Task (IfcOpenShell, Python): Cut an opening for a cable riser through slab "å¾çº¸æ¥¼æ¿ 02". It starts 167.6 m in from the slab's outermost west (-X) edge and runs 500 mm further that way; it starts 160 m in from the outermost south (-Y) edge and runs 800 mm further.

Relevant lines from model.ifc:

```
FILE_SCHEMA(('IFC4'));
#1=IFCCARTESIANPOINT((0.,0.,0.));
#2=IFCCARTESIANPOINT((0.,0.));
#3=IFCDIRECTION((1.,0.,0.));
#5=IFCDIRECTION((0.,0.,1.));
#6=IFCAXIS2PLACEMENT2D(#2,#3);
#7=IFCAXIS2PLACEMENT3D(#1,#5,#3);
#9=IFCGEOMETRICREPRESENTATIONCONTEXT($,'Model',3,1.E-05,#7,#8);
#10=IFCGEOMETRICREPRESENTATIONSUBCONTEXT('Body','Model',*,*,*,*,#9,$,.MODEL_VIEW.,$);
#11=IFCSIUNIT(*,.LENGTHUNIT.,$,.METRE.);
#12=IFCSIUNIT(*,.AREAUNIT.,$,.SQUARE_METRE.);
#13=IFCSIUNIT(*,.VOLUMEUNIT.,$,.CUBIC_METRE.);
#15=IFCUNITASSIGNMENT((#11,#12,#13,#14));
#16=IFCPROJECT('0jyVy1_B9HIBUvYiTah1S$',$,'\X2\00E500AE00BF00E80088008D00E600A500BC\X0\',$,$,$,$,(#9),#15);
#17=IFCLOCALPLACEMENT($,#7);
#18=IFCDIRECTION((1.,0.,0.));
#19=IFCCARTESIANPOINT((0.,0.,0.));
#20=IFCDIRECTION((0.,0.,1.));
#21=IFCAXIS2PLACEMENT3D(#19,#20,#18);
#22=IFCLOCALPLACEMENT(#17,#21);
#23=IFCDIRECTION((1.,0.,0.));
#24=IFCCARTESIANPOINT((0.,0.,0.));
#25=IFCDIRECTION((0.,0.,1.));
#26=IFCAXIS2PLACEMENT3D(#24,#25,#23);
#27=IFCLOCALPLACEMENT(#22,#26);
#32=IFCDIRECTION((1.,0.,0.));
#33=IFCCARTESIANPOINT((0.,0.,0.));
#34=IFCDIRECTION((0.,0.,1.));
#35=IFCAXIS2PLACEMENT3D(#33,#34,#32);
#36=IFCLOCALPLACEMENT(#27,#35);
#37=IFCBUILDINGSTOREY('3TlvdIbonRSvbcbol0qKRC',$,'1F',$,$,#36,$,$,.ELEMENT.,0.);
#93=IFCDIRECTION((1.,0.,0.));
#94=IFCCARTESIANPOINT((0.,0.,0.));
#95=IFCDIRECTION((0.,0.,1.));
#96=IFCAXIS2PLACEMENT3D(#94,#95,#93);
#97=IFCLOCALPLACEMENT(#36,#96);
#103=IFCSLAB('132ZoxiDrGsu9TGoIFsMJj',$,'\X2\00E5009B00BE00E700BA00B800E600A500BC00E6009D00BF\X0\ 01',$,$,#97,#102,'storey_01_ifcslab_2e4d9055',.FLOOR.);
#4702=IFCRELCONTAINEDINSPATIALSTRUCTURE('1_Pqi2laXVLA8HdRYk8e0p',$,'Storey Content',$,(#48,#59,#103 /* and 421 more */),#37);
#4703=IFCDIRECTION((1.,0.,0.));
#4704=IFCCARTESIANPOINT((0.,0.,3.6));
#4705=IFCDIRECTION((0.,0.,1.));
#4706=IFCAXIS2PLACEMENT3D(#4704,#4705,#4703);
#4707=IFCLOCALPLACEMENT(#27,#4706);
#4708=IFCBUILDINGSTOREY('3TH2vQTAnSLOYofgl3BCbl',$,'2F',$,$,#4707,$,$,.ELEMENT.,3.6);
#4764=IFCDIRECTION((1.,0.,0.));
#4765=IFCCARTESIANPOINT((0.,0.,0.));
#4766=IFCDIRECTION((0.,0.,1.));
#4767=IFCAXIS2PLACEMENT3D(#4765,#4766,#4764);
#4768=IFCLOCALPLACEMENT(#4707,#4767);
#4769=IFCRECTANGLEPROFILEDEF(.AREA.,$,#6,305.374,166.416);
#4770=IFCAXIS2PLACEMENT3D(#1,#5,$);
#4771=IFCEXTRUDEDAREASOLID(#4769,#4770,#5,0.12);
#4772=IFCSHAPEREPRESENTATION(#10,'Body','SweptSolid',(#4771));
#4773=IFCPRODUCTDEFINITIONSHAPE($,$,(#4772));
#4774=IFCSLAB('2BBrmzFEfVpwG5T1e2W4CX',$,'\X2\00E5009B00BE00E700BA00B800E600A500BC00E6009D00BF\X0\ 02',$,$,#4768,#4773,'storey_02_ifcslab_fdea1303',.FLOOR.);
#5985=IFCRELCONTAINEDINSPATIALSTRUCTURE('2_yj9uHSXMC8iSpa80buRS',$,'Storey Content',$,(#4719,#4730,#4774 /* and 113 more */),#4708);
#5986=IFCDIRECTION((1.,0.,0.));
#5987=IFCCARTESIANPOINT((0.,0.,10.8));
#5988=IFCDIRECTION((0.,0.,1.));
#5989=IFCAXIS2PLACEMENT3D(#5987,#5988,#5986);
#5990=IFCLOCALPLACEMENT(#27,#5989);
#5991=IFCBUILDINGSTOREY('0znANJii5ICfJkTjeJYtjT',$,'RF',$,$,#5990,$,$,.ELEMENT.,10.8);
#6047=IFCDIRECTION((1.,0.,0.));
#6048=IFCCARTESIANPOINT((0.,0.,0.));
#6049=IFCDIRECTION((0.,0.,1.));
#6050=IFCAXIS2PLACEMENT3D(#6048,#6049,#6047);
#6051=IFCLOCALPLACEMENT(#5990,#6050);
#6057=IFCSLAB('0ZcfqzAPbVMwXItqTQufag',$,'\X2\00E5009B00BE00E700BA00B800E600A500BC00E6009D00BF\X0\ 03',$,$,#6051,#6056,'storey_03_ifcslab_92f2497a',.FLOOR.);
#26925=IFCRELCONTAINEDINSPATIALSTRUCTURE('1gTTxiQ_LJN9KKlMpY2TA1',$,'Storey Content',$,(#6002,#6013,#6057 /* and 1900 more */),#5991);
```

```python
import numpy as np
import ifcopenshell
import ifcopenshell.api.feature
import ifcopenshell.api.geometry
import ifcopenshell.api.root
import ifcopenshell.geom
import ifcopenshell.util.placement
import ifcopenshell.util.representation
import ifcopenshell.util.shape
import ifcopenshell.util.unit

model = ifcopenshell.open("model.ifc")
unit_scale = ifcopenshell.util.unit.calculate_unit_scale(model)
settings = ifcopenshell.geom.settings()


def volume(element):
    """Net volume in cubic metres, openings subtracted."""
    shape = ifcopenshell.geom.create_shape(settings, element)
    return ifcopenshell.util.shape.get_volume(shape.geometry)


slab = model.by_guid("2BBrmzFEfVpwG5T1e2W4CX")
before = volume(slab)

# Extent in the slab's own axes, in metres. The edges named are its -X and -Y sides.
slab_shape = ifcopenshell.geom.create_shape(settings, slab)
vertices = ifcopenshell.util.shape.get_vertices(slab_shape.geometry)
x_min, y_min, bottom = vertices.min(axis=0)
top = vertices[:, 2].max()

opening = ifcopenshell.api.root.create_entity(model, ifc_class="IfcOpeningElement", name="Cable riser opening", predefined_type="OPENING")
context = ifcopenshell.util.representation.get_context(model, "Model", "Body", "MODEL_VIEW")
width, depth = 0.5, 0.8
outline = [(0.0, 0.0), (width, 0.0), (width, depth), (0.0, depth), (0.0, 0.0)]
# Overshoot both faces by 50 mm so the cut is clean.
shape = ifcopenshell.api.geometry.add_slab_representation(
    model, context=context, depth=top - bottom + 0.1, polyline=outline
)
ifcopenshell.api.geometry.assign_representation(model, product=opening, representation=shape)

matrix = ifcopenshell.util.placement.get_local_placement(slab.ObjectPlacement)
matrix[:, 3] = matrix @ np.append(np.array([x_min + 167.6, y_min + 160, bottom - 0.05]) / unit_scale, 1.0)
ifcopenshell.api.geometry.edit_object_placement(model, product=opening, matrix=matrix, is_si=False)
ifcopenshell.api.feature.add_feature(model, feature=opening, element=slab)

after = volume(slab)

print(f"slab volume {before:.3f} -> {after:.3f} m3")

model.write("model_v2.ifc")
```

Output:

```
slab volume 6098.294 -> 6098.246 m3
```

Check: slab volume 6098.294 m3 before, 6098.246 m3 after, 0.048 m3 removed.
